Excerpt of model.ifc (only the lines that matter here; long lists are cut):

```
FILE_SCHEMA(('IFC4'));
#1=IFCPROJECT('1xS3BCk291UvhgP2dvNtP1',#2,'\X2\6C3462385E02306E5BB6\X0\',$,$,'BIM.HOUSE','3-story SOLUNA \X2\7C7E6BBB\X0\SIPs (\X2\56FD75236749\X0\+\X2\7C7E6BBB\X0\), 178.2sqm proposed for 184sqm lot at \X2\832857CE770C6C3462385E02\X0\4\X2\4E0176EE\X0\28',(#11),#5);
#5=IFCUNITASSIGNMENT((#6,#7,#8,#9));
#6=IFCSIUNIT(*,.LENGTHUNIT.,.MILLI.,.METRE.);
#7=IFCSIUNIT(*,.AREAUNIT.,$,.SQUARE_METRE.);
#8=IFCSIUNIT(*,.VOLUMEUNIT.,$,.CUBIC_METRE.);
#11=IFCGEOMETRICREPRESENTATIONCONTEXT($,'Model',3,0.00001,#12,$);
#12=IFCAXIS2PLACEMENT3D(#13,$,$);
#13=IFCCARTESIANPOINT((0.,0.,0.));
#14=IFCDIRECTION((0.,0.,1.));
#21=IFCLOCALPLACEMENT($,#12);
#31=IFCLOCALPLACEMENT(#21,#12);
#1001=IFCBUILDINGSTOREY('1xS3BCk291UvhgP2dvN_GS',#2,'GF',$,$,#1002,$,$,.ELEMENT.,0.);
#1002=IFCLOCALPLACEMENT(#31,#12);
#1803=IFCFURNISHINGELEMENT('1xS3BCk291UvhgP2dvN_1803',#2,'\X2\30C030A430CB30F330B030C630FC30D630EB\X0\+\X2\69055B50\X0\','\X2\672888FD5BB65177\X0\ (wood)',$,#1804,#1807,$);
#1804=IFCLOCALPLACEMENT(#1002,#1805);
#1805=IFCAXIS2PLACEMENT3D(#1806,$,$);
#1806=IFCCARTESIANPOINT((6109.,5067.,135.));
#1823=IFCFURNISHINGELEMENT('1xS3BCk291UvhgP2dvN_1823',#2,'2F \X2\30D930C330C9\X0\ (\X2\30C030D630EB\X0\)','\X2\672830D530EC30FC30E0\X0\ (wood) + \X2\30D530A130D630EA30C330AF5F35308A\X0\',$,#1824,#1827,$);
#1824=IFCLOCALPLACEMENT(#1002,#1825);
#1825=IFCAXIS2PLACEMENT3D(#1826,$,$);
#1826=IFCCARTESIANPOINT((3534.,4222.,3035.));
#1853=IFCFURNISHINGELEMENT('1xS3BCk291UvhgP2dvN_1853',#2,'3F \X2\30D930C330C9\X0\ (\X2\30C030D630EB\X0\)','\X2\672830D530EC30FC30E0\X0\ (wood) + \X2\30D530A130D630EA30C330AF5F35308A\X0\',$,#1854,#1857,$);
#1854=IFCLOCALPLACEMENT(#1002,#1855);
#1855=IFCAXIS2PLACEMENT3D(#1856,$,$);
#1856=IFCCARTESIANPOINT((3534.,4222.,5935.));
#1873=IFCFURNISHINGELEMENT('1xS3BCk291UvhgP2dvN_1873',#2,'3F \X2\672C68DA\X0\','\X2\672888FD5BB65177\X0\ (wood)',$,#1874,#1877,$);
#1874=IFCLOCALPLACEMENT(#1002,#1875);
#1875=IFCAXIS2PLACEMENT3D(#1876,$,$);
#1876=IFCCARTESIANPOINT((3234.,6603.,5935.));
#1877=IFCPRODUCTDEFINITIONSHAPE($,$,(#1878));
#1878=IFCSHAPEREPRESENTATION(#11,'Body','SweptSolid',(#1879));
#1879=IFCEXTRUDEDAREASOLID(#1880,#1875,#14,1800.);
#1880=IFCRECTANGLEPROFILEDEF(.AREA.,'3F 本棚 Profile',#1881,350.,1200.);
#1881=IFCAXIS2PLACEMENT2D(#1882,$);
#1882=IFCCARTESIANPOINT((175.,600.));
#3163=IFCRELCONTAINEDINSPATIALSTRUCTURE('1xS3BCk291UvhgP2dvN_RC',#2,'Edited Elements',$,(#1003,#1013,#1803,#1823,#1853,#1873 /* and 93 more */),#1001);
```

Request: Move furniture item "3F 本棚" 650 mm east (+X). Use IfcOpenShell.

```python
import ifcopenshell
import ifcopenshell.api.geometry
import ifcopenshell.util.placement

model = ifcopenshell.open("model.ifc")

item = model.by_guid("1xS3BCk291UvhgP2dvN_1873")
matrix = ifcopenshell.util.placement.get_local_placement(item.ObjectPlacement)
matrix[0, 3] += 650.0
ifcopenshell.api.geometry.edit_object_placement(model, product=item, matrix=matrix, is_si=False)

print(ifcopenshell.util.placement.get_local_placement(item.ObjectPlacement).round(3) + 0.0)

model.write("model_rev.ifc")
```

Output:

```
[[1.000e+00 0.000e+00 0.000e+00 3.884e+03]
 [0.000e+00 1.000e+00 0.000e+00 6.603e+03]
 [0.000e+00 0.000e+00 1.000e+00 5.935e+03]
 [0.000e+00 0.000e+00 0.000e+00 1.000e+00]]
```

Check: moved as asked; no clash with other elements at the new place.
